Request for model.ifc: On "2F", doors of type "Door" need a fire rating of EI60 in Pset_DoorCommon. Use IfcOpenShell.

First a look at what the model holds.

```python
import ifcopenshell
import ifcopenshell.util.element

model = ifcopenshell.open("model.ifc")
print(model.schema)
storey = next(s for s in model.by_type("IfcBuildingStorey") if s.Name == "2F")
doors = [e for e in ifcopenshell.util.element.get_decomposition(storey) if e.is_a("IfcDoor")]
seen = {}
for e in doors:
    element_type = ifcopenshell.util.element.get_type(e)
    key = (element_type.Name if element_type != e and element_type else None, ifcopenshell.util.element.get_pset(e, "Pset_DoorCommon", "FireRating"))
    seen[key] = seen.get(key, 0) + 1
for (name, value), count in sorted(seen.items(), key=str):
    print(count, "x", name, "|", value)
```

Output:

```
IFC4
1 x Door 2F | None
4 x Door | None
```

```python
import ifcopenshell
import ifcopenshell.api.pset
import ifcopenshell.util.element

model = ifcopenshell.open("model.ifc")

storey = next(s for s in model.by_type("IfcBuildingStorey") if s.Name == "2F")
doors = [e for e in ifcopenshell.util.element.get_decomposition(storey) if e.is_a("IfcDoor")]

count = 0
for e in doors:
    element_type = ifcopenshell.util.element.get_type(e)
    if element_type in (None, e) or element_type.Name != "Door":
        continue
    # add_pset returns the element's existing set when there is one.
    pset = ifcopenshell.api.pset.add_pset(model, product=e, name="Pset_DoorCommon")
    ifcopenshell.api.pset.edit_pset(model, pset=pset, properties={"FireRating": "EI60"})
    count += 1

print(count, "doors updated")

model.write("model_updated.ifc")
```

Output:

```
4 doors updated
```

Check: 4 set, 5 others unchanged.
